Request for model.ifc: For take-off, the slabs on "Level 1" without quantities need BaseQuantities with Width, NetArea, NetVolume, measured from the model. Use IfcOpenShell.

First a look at what the model holds.

```python
import ifcopenshell
import ifcopenshell.util.element
import ifcopenshell.util.unit

model = ifcopenshell.open("model.ifc")
print(model.schema)
for unit_type in ("LENGTHUNIT", "AREAUNIT", "VOLUMEUNIT"):
    print(unit_type, ifcopenshell.util.unit.calculate_unit_scale(model, unit_type))
storey = next(s for s in model.by_type("IfcBuildingStorey") if s.Name == "Level 1")
slabs = [e for e in ifcopenshell.util.element.get_decomposition(storey) if e.is_a("IfcSlab")]
for e in sorted(slabs, key=lambda e: e.id()):
    print(e.id(), e.is_a(), e.Name, list(ifcopenshell.util.element.get_psets(e, qtos_only=True)), sep=" | ")
```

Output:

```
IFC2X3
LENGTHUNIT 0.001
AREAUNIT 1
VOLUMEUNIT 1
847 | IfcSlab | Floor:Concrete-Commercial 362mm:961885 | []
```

```python
import ifcopenshell
import ifcopenshell.api.pset
import ifcopenshell.geom
import ifcopenshell.util.element
import ifcopenshell.util.shape
import ifcopenshell.util.unit

model = ifcopenshell.open("model.ifc")
unit_scale = ifcopenshell.util.unit.calculate_unit_scale(model)
area_scale = ifcopenshell.util.unit.calculate_unit_scale(model, "AREAUNIT")
volume_scale = ifcopenshell.util.unit.calculate_unit_scale(model, "VOLUMEUNIT")
settings = ifcopenshell.geom.settings()

storey = next(s for s in model.by_type("IfcBuildingStorey") if s.Name == "Level 1")
slabs = [e for e in ifcopenshell.util.element.get_decomposition(storey) if e.is_a("IfcSlab")]

for e in sorted(slabs, key=lambda e: e.id()):
    if ifcopenshell.util.element.get_psets(e, qtos_only=True, should_inherit=False):
        continue
    # Geometry comes back in metres, in the element's own axes.
    shape = ifcopenshell.geom.create_shape(settings, e)
    values = {
        "Width": ifcopenshell.util.shape.get_z(shape.geometry) / unit_scale,
        "NetArea": ifcopenshell.util.shape.get_footprint_area(shape.geometry) / area_scale,
        "NetVolume": ifcopenshell.util.shape.get_volume(shape.geometry) / volume_scale,
    }
    qto = ifcopenshell.api.pset.add_qto(model, product=e, name="BaseQuantities")
    ifcopenshell.api.pset.edit_qto(model, qto=qto, properties=values)
    print(e.id(), {k: round(v, 3) for k, v in values.items()})

model.write("model-out.ifc")
```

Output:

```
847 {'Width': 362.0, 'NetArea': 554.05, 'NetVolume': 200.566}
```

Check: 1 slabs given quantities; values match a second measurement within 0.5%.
